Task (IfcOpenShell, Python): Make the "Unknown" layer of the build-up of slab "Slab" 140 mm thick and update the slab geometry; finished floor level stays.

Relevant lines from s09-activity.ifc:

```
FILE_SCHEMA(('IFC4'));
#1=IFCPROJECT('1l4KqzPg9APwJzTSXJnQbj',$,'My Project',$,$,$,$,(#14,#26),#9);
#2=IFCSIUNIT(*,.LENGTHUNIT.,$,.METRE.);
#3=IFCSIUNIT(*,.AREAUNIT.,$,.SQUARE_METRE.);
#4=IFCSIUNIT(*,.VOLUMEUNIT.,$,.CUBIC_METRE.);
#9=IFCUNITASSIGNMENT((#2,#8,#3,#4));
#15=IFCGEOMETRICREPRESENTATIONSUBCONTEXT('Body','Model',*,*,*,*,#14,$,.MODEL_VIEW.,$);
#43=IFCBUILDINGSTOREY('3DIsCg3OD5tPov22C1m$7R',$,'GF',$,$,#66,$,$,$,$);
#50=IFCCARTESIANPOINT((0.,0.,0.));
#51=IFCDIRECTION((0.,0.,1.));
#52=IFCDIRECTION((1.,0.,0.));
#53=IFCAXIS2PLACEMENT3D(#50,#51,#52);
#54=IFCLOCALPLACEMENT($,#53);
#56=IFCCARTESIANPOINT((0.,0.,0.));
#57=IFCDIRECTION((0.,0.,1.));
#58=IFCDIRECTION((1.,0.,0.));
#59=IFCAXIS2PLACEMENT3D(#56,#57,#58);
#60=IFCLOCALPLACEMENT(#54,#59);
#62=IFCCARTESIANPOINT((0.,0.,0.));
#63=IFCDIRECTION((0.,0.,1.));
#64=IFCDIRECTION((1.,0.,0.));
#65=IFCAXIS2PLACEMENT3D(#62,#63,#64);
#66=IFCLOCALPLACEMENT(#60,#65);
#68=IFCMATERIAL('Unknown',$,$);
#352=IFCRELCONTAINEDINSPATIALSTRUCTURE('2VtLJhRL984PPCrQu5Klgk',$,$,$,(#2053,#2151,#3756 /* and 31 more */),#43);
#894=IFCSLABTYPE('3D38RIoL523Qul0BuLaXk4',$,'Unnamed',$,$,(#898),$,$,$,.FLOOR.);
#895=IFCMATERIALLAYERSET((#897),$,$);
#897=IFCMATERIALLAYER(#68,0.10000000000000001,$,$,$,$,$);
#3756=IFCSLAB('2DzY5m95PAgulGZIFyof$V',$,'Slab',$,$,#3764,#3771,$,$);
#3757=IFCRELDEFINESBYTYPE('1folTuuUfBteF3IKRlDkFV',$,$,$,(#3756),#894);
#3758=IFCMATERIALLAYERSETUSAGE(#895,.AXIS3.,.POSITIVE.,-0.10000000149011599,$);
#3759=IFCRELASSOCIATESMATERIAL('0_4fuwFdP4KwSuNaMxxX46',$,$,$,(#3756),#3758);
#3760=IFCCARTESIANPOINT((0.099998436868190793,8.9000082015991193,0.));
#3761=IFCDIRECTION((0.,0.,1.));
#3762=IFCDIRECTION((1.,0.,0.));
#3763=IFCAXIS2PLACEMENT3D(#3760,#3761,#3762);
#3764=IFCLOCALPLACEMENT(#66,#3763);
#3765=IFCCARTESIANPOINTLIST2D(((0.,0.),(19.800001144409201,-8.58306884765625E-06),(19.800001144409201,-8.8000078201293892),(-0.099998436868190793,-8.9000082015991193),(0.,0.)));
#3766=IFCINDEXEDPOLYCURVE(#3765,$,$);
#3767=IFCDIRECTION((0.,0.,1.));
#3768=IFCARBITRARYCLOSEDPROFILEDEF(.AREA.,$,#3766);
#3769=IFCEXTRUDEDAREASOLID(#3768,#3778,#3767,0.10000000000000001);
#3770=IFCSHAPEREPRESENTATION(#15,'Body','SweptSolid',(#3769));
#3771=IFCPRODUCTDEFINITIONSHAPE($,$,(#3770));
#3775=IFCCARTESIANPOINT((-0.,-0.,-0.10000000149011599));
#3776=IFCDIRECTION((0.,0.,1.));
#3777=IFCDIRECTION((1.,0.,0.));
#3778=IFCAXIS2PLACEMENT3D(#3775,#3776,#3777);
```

```python
import ifcopenshell
import ifcopenshell.util.element
import ifcopenshell.util.representation

model = ifcopenshell.open("s09-activity.ifc")

layer_set = model.by_id(895)
layer = next(l for l in layer_set.MaterialLayers if l.Material and l.Material.Name == "Unknown")
change = 0.14 - layer.LayerThickness
layer.LayerThickness += change

# Geometry does not follow the layer set by itself.
slabs = [e for e in ifcopenshell.util.element.get_elements_by_material(model, layer_set) if e.is_a("IfcSlab")]
for slab in sorted(slabs, key=lambda e: e.id()):
    body = ifcopenshell.util.representation.get_representation(slab, "Model", "Body")
    solid = body.Items[0]
    old_depth = solid.Depth
    solid.Depth += change
    # Extruded upwards: lower the start of the extrusion so the top stays.
    x, y, z = solid.Position.Location.Coordinates
    solid.Position.Location = model.createIfcCartesianPoint((x, y, z - change))
    print(slab.id(), f"{old_depth:g} -> {solid.Depth:g}")

# The layers are counted up from the underside, which has moved.
for usage in {ifcopenshell.util.element.get_material(slab) for slab in slabs}:
    usage.OffsetFromReferenceLine -= change

model.write("s09-activity_rev.ifc")
```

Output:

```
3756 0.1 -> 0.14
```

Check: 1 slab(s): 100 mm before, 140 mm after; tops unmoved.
